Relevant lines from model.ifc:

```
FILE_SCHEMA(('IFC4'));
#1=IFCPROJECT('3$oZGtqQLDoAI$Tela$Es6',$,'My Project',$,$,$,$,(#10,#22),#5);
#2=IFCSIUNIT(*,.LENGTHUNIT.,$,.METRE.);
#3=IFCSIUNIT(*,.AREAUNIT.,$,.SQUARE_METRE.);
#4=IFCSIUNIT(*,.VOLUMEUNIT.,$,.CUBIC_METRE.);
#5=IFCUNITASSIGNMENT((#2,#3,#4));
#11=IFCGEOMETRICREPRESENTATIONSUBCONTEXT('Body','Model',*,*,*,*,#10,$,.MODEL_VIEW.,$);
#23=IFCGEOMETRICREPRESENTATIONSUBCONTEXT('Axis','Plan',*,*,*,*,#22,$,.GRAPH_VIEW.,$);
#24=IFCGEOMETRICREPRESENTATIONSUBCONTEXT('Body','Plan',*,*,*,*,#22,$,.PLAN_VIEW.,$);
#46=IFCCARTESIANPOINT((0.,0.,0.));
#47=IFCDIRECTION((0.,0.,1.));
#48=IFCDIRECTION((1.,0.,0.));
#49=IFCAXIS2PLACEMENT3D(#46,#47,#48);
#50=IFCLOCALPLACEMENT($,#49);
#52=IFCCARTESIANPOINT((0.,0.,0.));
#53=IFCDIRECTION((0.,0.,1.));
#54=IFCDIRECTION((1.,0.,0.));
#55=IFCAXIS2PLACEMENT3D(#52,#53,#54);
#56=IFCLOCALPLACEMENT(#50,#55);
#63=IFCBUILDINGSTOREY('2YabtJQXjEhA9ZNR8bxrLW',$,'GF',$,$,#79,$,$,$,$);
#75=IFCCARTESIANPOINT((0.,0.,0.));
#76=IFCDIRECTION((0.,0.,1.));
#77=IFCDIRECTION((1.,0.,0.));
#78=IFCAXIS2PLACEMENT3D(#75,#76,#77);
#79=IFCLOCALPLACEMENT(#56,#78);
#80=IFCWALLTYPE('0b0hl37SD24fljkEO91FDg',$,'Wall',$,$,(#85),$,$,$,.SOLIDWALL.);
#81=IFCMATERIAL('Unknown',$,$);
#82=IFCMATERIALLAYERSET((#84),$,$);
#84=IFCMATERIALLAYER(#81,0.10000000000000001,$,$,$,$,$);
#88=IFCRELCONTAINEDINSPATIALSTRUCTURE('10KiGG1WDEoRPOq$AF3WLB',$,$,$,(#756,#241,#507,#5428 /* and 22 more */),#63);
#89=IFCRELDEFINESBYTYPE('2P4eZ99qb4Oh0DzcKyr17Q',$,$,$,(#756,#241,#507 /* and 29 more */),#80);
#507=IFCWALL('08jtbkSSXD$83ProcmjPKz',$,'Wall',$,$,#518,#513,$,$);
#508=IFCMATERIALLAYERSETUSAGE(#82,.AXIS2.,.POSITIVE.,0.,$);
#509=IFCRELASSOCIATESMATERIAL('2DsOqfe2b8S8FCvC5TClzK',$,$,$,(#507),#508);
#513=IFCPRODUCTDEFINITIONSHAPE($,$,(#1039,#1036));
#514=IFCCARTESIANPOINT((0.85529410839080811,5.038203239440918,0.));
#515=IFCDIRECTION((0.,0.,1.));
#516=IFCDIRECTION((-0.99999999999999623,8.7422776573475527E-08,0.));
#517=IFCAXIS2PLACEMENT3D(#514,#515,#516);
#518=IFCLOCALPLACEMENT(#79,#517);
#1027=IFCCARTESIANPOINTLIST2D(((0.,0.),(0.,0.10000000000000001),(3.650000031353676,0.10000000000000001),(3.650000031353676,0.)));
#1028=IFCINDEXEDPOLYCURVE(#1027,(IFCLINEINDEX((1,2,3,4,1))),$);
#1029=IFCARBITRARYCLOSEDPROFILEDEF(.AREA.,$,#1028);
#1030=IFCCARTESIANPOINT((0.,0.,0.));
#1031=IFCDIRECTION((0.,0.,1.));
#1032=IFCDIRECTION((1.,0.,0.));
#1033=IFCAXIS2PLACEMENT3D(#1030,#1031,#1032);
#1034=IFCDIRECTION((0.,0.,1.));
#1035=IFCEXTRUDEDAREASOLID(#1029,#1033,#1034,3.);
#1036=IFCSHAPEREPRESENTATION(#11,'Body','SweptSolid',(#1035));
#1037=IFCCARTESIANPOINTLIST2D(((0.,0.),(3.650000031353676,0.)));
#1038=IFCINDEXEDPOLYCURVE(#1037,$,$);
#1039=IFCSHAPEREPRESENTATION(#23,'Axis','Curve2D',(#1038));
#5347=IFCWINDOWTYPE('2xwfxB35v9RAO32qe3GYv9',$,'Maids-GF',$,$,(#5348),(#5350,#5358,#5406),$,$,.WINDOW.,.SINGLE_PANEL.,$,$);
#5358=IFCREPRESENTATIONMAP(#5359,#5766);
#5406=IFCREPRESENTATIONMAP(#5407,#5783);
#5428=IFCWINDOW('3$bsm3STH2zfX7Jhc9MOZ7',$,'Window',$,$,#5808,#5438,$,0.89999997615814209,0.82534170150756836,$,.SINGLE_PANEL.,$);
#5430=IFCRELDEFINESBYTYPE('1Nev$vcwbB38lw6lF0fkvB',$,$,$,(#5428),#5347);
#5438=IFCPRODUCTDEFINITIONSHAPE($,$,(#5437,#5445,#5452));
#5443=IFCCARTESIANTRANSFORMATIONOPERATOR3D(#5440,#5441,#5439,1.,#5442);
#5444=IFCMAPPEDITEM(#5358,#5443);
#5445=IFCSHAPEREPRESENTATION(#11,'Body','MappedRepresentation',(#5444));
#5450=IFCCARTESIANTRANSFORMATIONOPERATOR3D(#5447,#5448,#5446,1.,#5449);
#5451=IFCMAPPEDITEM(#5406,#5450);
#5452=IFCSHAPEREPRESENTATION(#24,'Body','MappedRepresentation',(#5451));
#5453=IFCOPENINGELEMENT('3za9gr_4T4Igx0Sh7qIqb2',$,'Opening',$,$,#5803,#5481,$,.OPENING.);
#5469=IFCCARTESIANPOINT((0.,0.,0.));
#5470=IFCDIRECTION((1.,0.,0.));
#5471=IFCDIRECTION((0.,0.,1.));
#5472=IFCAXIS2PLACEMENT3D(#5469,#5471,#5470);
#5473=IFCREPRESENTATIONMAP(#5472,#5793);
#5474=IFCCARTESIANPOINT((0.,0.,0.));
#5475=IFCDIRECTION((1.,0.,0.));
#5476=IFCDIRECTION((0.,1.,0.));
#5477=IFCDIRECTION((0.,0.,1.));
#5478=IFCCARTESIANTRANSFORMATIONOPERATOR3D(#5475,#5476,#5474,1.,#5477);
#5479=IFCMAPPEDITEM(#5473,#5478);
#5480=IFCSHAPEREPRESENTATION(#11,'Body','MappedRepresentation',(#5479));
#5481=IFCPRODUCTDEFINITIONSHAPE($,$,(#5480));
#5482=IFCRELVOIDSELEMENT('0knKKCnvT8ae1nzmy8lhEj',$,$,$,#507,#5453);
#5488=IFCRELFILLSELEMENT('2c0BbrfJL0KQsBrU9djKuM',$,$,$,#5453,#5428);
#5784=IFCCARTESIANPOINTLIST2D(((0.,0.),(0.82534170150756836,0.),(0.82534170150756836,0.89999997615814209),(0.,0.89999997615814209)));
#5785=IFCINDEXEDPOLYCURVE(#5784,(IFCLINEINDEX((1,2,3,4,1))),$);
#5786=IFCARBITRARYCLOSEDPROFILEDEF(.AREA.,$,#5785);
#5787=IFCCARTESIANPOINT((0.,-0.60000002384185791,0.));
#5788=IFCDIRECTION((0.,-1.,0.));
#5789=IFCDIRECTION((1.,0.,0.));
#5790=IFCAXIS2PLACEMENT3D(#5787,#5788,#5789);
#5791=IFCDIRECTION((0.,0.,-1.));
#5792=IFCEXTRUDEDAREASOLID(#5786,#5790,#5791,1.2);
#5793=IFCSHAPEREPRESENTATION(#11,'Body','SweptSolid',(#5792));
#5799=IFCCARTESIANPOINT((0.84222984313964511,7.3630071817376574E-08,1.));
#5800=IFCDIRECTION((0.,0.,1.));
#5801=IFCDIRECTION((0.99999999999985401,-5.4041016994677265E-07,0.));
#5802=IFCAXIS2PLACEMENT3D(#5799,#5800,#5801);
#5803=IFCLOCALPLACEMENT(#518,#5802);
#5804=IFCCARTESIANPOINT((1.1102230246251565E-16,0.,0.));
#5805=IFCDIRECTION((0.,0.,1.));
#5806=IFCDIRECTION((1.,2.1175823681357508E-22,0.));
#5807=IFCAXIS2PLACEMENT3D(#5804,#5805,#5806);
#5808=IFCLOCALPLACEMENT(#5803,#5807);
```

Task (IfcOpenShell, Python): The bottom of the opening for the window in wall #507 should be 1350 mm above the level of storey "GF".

```python
import numpy as np
import ifcopenshell
import ifcopenshell.api.geometry
import ifcopenshell.geom
import ifcopenshell.util.element
import ifcopenshell.util.placement
import ifcopenshell.util.shape
import ifcopenshell.util.unit

model = ifcopenshell.open("model.ifc")
unit_scale = ifcopenshell.util.unit.calculate_unit_scale(model)

window = model.by_id(5428)
opening = window.FillsVoids[0].RelatingOpeningElement
storey = ifcopenshell.util.element.get_container(window, ifc_class="IfcBuildingStorey")
level = ifcopenshell.util.placement.get_local_placement(storey.ObjectPlacement)[2, 3]

# The opening's origin need not be at the sill, so measure its lowest point.
shape = ifcopenshell.geom.create_shape(ifcopenshell.geom.settings(), opening)
bottom = ifcopenshell.util.shape.get_shape_bottom_elevation(shape, shape.geometry) / unit_scale
dz = level + 1.35 - bottom

shift = np.array([0.0, 0.0, dz])
# The window is placed relative to its opening, so it follows when the opening moves.
matrix = ifcopenshell.util.placement.get_local_placement(opening.ObjectPlacement)
matrix[:3, 3] += shift
ifcopenshell.api.geometry.edit_object_placement(
    model, product=opening, matrix=matrix, is_si=False, should_transform_children=True
)

print(f"moved by {dz * unit_scale:+.3f} m")

model.write("model_edited.ifc")
```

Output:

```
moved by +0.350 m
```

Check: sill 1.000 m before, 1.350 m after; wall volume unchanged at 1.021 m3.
